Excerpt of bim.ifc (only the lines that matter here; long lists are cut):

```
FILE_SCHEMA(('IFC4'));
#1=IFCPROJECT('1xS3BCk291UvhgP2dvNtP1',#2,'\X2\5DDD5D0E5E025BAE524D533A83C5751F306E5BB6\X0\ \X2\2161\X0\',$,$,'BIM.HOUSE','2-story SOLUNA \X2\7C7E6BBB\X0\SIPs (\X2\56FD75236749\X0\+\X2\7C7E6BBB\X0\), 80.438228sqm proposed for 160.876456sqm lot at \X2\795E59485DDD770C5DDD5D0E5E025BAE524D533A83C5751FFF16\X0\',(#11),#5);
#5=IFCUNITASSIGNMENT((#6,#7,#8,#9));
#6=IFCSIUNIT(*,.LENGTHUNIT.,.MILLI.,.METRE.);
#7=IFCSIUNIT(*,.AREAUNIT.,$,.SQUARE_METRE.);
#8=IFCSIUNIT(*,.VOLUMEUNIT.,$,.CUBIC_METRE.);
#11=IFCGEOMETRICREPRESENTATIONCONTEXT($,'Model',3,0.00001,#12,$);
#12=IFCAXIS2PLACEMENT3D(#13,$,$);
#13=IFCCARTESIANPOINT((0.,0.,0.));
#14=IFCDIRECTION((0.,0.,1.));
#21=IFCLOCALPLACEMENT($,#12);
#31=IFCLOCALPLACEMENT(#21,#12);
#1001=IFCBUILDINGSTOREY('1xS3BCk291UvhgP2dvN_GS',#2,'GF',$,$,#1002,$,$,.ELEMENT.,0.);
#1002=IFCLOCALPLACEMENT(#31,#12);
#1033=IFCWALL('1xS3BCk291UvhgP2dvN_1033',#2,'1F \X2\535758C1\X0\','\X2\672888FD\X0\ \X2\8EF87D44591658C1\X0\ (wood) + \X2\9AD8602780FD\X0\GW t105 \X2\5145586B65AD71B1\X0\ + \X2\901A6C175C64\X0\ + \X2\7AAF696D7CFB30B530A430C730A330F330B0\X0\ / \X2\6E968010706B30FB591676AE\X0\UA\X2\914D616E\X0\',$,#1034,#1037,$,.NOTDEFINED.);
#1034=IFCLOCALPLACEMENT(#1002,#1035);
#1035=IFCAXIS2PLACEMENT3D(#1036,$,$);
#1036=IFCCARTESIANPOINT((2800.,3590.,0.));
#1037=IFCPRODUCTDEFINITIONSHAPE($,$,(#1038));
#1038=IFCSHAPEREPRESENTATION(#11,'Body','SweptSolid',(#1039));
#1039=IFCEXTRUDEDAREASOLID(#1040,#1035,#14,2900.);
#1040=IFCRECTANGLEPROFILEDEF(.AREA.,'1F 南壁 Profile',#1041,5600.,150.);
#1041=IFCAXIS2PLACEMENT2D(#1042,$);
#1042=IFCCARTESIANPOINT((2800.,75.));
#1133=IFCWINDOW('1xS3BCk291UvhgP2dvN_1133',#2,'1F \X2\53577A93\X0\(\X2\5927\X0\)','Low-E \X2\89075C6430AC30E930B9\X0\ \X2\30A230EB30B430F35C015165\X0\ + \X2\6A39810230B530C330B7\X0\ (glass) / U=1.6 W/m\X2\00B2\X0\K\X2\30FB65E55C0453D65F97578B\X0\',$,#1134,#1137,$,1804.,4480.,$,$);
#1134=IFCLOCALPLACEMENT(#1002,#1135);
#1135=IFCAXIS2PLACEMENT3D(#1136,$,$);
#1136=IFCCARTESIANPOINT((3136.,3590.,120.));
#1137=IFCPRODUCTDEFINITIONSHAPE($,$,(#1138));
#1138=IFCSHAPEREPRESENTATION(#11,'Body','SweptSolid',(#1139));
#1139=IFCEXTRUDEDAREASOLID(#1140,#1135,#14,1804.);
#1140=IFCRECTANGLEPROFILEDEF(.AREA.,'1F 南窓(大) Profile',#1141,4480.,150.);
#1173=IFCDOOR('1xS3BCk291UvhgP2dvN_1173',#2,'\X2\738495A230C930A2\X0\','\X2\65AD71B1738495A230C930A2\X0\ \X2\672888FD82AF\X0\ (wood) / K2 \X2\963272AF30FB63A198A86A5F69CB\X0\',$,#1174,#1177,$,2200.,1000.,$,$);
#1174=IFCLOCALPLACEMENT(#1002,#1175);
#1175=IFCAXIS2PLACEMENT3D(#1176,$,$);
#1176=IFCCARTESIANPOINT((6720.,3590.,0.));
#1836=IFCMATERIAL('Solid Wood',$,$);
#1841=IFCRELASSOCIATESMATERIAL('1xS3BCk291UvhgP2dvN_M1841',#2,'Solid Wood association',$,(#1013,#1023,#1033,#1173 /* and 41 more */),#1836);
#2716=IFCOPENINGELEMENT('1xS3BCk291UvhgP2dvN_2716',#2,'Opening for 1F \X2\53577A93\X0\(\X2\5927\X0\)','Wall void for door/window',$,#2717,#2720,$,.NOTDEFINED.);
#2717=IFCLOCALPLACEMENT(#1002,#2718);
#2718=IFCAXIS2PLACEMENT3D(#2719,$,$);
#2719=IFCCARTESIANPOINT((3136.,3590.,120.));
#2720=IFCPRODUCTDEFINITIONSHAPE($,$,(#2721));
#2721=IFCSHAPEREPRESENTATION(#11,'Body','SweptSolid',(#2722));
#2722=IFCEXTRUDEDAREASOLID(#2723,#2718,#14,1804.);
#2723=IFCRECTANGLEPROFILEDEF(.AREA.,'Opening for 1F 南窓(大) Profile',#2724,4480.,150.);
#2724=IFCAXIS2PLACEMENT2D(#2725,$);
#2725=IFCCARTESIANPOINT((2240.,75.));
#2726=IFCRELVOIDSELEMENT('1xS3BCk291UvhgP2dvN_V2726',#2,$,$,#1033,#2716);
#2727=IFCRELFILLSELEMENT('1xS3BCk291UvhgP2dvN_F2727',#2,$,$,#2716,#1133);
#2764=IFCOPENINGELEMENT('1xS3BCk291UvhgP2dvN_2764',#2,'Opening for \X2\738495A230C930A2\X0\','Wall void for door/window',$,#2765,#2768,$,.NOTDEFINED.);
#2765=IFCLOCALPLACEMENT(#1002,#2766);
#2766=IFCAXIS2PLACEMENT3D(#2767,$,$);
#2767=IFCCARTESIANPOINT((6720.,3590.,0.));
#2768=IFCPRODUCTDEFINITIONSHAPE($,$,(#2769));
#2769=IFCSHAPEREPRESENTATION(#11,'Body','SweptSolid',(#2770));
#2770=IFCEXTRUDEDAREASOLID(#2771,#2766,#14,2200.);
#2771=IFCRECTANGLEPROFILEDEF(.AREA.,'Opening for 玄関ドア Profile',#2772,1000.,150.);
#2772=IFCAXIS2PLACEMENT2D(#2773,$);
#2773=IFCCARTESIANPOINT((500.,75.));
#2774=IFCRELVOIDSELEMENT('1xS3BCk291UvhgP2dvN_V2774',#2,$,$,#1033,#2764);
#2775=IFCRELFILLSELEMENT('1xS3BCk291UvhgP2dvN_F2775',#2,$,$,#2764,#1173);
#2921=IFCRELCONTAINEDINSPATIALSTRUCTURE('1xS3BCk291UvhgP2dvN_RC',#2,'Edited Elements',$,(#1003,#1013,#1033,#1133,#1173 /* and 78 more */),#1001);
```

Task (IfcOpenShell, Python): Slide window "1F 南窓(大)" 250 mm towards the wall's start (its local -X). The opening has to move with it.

```python
import ifcopenshell
import ifcopenshell.api.geometry
import ifcopenshell.util.placement
import ifcopenshell.util.unit

model = ifcopenshell.open("bim.ifc")
unit_scale = ifcopenshell.util.unit.calculate_unit_scale(model)

window = model.by_guid("1xS3BCk291UvhgP2dvN_1133")
opening = window.FillsVoids[0].RelatingOpeningElement
wall = opening.VoidsElements[0].RelatingBuildingElement

wall_matrix = ifcopenshell.util.placement.get_local_placement(wall.ObjectPlacement)
shift = wall_matrix[:3, 0] * -0.25 / unit_scale
before = ifcopenshell.util.placement.get_local_placement(window.ObjectPlacement)[:3, 3].copy()

# The window is not placed relative to its opening, so move both.
for product in (opening, window):
    matrix = ifcopenshell.util.placement.get_local_placement(product.ObjectPlacement)
    matrix[:3, 3] += shift
    ifcopenshell.api.geometry.edit_object_placement(model, product=product, matrix=matrix, is_si=False)

after = ifcopenshell.util.placement.get_local_placement(window.ObjectPlacement)[:3, 3]
print("window moved by", (after - before).round(3) + 0.0)

model.write("bim_v2.ifc")
```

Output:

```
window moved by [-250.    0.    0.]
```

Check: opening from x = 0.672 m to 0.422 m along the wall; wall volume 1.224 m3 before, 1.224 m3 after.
